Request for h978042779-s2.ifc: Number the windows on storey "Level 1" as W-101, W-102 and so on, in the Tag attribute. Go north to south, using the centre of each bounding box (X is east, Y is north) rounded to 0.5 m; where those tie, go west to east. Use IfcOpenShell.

First a look at what the model holds.

```python
import ifcopenshell
import ifcopenshell.util.element
import ifcopenshell.util.placement

model = ifcopenshell.open("h978042779-s2.ifc")
print(model.schema)
storey = next(s for s in model.by_type("IfcBuildingStorey") if s.Name == "Level 1")
windows = [e for e in ifcopenshell.util.element.get_decomposition(storey) if e.is_a("IfcWindow")]
for e in sorted(windows, key=lambda e: e.id()):
    origin = ifcopenshell.util.placement.get_local_placement(e.ObjectPlacement)[:3, 3]
    print(e.id(), e.Tag, e.Name, origin.round(2) + 0.0, sep=" | ")
```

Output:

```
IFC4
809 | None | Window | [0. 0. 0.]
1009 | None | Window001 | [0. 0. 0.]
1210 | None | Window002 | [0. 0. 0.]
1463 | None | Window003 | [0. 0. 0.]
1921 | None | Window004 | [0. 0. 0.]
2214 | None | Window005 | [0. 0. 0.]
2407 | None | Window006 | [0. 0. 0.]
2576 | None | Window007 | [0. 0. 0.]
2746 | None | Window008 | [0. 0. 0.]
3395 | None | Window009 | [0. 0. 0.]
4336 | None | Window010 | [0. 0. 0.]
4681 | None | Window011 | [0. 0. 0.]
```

```python
import ifcopenshell
import ifcopenshell.geom
import ifcopenshell.util.element
import ifcopenshell.util.shape

model = ifcopenshell.open("h978042779-s2.ifc")
settings = ifcopenshell.geom.settings()
settings.set("use-world-coords", True)


def centre(element):
    shape = ifcopenshell.geom.create_shape(settings, element)
    return ifcopenshell.util.shape.get_bbox_centroid(shape.geometry)


storey = next(s for s in model.by_type("IfcBuildingStorey") if s.Name == "Level 1")
windows = [e for e in ifcopenshell.util.element.get_decomposition(storey) if e.is_a("IfcWindow")]

# Insertion points can sit at a corner or the storey origin, so sort by the geometry (in metres).
centres = {e: centre(e) for e in windows}
windows.sort(key=lambda e: (-round(centres[e][1] / 0.5), centres[e][0]))

for i, e in enumerate(windows, start=1):
    number = f"W-1{i:02d}"
    e.Tag = number
    print(e.id(), number)

model.write("h978042779-s2-out.ifc")
```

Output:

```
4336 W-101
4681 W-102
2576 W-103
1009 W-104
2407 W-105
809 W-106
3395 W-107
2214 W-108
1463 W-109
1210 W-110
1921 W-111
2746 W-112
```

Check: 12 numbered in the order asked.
